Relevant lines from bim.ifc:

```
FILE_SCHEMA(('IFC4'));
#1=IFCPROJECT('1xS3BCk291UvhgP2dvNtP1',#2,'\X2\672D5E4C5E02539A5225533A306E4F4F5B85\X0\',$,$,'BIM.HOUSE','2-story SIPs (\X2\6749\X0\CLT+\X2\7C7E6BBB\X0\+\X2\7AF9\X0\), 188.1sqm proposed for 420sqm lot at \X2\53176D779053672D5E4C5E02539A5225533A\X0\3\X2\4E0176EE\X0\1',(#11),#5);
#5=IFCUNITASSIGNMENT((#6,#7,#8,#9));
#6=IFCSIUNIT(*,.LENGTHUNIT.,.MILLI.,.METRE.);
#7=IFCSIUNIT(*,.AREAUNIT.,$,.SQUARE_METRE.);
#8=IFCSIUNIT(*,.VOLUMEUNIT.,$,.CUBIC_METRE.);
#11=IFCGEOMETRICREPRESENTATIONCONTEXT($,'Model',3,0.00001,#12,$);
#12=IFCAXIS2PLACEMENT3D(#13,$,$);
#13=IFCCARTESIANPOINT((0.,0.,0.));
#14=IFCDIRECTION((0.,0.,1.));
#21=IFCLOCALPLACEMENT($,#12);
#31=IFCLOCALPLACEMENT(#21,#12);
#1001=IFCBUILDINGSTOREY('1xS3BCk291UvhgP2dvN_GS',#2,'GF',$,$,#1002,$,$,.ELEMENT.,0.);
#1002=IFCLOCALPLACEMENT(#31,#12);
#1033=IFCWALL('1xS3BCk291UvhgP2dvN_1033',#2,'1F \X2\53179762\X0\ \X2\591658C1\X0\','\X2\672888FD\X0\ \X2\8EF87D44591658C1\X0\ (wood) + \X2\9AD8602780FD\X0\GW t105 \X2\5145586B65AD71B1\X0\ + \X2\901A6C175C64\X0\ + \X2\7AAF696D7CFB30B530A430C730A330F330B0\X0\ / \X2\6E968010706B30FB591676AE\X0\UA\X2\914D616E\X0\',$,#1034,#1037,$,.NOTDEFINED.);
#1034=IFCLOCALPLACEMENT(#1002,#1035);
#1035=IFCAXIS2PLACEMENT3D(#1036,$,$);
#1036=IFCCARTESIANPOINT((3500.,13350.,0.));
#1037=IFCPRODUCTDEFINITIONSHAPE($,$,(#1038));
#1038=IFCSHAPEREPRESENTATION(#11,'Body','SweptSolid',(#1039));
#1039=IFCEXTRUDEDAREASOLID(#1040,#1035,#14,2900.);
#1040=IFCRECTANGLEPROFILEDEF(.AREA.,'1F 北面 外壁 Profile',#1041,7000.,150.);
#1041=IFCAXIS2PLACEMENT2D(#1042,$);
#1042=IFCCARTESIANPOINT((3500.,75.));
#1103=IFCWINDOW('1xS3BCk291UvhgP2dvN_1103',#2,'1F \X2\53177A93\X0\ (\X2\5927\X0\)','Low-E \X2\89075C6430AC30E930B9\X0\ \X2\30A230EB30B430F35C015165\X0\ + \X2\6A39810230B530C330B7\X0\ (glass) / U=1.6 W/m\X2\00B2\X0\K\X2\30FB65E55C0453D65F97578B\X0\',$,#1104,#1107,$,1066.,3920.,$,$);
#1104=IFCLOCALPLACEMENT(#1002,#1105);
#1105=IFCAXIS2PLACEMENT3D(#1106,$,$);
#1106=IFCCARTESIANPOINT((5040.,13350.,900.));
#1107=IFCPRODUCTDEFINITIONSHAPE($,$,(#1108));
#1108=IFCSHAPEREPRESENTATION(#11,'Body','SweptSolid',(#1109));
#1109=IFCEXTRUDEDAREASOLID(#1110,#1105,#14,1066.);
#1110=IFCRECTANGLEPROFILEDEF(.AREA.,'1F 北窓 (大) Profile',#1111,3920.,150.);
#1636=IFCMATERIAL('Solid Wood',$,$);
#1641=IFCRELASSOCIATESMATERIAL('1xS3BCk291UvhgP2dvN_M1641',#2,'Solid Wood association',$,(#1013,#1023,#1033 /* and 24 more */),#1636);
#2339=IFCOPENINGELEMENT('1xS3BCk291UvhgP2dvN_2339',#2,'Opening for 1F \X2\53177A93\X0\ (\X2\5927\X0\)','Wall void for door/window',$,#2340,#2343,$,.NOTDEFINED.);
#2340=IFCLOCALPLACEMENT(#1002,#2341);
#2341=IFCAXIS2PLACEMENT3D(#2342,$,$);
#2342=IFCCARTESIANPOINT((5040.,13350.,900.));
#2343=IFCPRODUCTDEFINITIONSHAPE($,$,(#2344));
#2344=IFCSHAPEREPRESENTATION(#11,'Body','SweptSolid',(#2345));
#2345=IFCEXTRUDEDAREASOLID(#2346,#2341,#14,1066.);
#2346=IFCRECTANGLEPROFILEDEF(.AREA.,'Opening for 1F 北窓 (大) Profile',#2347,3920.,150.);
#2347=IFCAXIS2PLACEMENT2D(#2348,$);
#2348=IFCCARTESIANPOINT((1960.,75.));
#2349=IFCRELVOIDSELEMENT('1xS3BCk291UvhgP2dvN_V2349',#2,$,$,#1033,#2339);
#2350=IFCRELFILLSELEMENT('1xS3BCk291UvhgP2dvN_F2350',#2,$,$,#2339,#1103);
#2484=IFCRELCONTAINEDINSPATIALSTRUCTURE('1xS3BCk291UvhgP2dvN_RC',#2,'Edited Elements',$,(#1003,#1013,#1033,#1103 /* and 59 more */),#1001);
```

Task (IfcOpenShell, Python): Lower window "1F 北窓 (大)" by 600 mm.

```python
import numpy as np
import ifcopenshell
import ifcopenshell.api.geometry
import ifcopenshell.util.placement
import ifcopenshell.util.unit

model = ifcopenshell.open("bim.ifc")
unit_scale = ifcopenshell.util.unit.calculate_unit_scale(model)

window = model.by_id(1103)
opening = window.FillsVoids[0].RelatingOpeningElement
dz = -0.6 / unit_scale

shift = np.array([0.0, 0.0, dz])
# The window is not placed relative to its opening, so move both.
for product in (opening, window):
    matrix = ifcopenshell.util.placement.get_local_placement(product.ObjectPlacement)
    matrix[:3, 3] += shift
    ifcopenshell.api.geometry.edit_object_placement(model, product=product, matrix=matrix, is_si=False)

print(f"moved by {dz * unit_scale:+.3f} m")

model.write("bim-out.ifc")
```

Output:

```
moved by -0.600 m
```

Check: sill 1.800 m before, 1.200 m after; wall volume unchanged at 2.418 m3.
